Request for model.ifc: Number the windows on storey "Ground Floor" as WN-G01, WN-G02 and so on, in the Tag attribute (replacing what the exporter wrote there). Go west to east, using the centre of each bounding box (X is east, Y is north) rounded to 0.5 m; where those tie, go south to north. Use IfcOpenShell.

First a look at what the model holds.

```python
import ifcopenshell
import ifcopenshell.util.element
import ifcopenshell.util.placement

model = ifcopenshell.open("model.ifc")
print(model.schema)
storey = next(s for s in model.by_type("IfcBuildingStorey") if s.Name == "Ground Floor")
windows = [e for e in ifcopenshell.util.element.get_decomposition(storey) if e.is_a("IfcWindow")]
for e in sorted(windows, key=lambda e: e.id()):
    origin = ifcopenshell.util.placement.get_local_placement(e.ObjectPlacement)[:3, 3]
    print(e.id(), e.Tag, e.Name, origin.round(2) + 0.0, sep=" | ")
```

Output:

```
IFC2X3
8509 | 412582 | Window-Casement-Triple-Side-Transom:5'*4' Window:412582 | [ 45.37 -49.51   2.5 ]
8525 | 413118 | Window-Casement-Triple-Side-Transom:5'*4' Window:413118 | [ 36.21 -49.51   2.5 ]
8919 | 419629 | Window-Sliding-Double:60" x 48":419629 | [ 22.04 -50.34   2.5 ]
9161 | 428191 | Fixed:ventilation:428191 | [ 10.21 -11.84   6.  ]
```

```python
import ifcopenshell
import ifcopenshell.geom
import ifcopenshell.util.element
import ifcopenshell.util.shape

model = ifcopenshell.open("model.ifc")
settings = ifcopenshell.geom.settings()
settings.set("use-world-coords", True)


def centre(element):
    shape = ifcopenshell.geom.create_shape(settings, element)
    return ifcopenshell.util.shape.get_bbox_centroid(shape.geometry)


storey = next(s for s in model.by_type("IfcBuildingStorey") if s.Name == "Ground Floor")
windows = [e for e in ifcopenshell.util.element.get_decomposition(storey) if e.is_a("IfcWindow")]

# Insertion points can sit at a corner or the storey origin, so sort by the geometry (in metres).
centres = {e: centre(e) for e in windows}
windows.sort(key=lambda e: (round(centres[e][0] / 0.5), centres[e][1]))

for i, e in enumerate(windows, start=1):
    number = f"WN-G{i:02d}"
    e.Tag = number
    print(e.id(), number)

model.write("model-out.ifc")
```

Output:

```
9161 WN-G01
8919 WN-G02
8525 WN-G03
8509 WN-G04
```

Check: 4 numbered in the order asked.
